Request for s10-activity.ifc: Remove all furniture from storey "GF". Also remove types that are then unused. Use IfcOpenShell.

First a look at what the model holds.

```python
import ifcopenshell
import ifcopenshell.util.element

model = ifcopenshell.open("s10-activity.ifc")
print(model.schema)
storey = next(s for s in model.by_type("IfcBuildingStorey") if s.Name == "GF")
furniture = [e for e in ifcopenshell.util.element.get_decomposition(storey) if e.is_a("IfcFurnishingElement")]
seen = {}
for e in furniture:
    element_type = ifcopenshell.util.element.get_type(e)
    name = element_type.Name if element_type not in (None, e) else None
    seen[name] = seen.get(name, 0) + 1
for name, count in sorted(seen.items(), key=str):
    print(count, "x", name)
```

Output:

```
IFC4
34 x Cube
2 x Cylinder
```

```python
import ifcopenshell
import ifcopenshell.api.root
import ifcopenshell.util.element

model = ifcopenshell.open("s10-activity.ifc")

storey = next(s for s in model.by_type("IfcBuildingStorey") if s.Name == "GF")
furniture = [e for e in ifcopenshell.util.element.get_decomposition(storey) if e.is_a("IfcFurnishingElement")]
types = {ifcopenshell.util.element.get_type(e) for e in furniture} - {None, *furniture}

for e in furniture:
    ifcopenshell.api.root.remove_product(model, product=e)
print(len(furniture), "removed")

unused = [t for t in types if not ifcopenshell.util.element.get_types(t)]
for t in unused:
    ifcopenshell.api.root.remove_product(model, product=t)
print(len(unused), "unused types removed")

model.write("s10-activity_edited.ifc")
```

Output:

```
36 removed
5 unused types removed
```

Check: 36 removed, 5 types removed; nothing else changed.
